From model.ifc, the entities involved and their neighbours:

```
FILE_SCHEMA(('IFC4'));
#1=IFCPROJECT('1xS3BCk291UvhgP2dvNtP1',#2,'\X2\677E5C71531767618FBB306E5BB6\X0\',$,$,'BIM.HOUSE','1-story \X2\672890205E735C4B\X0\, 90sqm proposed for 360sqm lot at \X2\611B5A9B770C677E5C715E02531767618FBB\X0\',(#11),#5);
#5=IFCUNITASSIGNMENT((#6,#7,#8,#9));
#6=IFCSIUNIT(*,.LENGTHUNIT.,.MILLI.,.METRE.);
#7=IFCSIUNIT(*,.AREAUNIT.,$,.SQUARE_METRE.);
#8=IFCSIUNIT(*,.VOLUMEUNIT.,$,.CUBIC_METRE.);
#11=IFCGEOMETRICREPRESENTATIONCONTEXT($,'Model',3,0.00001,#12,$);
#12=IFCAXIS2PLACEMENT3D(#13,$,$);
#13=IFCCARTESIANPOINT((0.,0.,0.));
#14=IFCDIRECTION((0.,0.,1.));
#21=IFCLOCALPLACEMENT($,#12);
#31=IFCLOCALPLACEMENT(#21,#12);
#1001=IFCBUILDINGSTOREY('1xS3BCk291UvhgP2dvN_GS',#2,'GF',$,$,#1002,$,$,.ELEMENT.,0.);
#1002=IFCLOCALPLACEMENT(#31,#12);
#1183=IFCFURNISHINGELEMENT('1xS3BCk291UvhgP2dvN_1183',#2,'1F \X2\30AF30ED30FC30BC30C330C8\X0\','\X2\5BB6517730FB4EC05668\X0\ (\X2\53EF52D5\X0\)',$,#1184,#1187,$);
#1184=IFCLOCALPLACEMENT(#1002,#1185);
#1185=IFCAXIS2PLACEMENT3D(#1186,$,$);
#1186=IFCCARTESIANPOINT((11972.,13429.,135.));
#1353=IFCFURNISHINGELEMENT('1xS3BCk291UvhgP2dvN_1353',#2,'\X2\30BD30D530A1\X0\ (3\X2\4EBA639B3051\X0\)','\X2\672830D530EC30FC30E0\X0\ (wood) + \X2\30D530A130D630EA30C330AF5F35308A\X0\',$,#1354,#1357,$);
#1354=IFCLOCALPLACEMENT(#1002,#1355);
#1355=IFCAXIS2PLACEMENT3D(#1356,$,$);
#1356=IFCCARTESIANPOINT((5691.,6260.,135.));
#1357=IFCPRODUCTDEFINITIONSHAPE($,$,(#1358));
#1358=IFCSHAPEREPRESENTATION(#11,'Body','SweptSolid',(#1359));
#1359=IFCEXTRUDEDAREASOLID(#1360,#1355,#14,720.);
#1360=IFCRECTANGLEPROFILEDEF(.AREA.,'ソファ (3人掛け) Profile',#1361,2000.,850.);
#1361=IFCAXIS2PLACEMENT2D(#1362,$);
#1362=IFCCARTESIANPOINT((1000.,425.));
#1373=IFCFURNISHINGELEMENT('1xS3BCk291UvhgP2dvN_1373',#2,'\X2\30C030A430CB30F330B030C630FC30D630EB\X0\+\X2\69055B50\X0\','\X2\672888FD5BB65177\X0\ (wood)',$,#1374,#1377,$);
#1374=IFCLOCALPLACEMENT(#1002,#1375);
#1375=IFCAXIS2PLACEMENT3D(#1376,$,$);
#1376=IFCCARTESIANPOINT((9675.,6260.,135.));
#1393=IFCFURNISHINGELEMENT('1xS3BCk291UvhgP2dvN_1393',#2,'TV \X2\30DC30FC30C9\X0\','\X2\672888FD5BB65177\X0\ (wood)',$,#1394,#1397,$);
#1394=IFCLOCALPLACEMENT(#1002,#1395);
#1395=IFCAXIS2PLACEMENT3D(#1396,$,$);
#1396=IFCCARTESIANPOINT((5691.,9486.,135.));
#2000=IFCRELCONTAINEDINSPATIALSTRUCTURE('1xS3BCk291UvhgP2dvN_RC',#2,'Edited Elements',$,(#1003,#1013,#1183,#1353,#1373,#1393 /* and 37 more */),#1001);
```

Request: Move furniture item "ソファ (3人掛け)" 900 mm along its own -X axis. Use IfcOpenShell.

```python
import ifcopenshell
import ifcopenshell.api.geometry
import ifcopenshell.util.placement
import ifcopenshell.util.unit

model = ifcopenshell.open("model.ifc")
unit_scale = ifcopenshell.util.unit.calculate_unit_scale(model)

item = model.by_guid("1xS3BCk291UvhgP2dvN_1353")
matrix = ifcopenshell.util.placement.get_local_placement(item.ObjectPlacement)
matrix[:3, 3] -= matrix[:3, 0] * 0.9 / unit_scale
ifcopenshell.api.geometry.edit_object_placement(model, product=item, matrix=matrix, is_si=False)

print(ifcopenshell.util.placement.get_local_placement(item.ObjectPlacement).round(3) + 0.0)

model.write("model_rev.ifc")
```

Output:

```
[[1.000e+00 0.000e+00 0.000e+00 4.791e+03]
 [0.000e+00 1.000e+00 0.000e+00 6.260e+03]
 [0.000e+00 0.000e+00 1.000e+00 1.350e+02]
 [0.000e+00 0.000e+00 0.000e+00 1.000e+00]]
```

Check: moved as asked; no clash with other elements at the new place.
